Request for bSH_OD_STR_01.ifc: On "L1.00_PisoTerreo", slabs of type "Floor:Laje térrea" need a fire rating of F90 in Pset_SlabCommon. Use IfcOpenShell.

First a look at what the model holds.

```python
import ifcopenshell
import ifcopenshell.util.element

model = ifcopenshell.open("bSH_OD_STR_01.ifc")
print(model.schema)
storey = next(s for s in model.by_type("IfcBuildingStorey") if s.Name == "L1.00_PisoTerreo")
slabs = [e for e in ifcopenshell.util.element.get_decomposition(storey) if e.is_a("IfcSlab")]
seen = {}
for e in slabs:
    element_type = ifcopenshell.util.element.get_type(e)
    key = (element_type.Name if element_type != e and element_type else None, ifcopenshell.util.element.get_pset(e, "Pset_SlabCommon", "FireRating"))
    seen[key] = seen.get(key, 0) + 1
for (name, value), count in sorted(seen.items(), key=str):
    print(count, "x", name, "|", value)
```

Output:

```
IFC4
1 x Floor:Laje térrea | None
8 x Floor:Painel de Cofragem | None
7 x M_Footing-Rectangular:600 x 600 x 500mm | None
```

```python
import ifcopenshell
import ifcopenshell.api.pset
import ifcopenshell.util.element

model = ifcopenshell.open("bSH_OD_STR_01.ifc")

storey = next(s for s in model.by_type("IfcBuildingStorey") if s.Name == "L1.00_PisoTerreo")
slabs = [e for e in ifcopenshell.util.element.get_decomposition(storey) if e.is_a("IfcSlab")]

count = 0
for e in slabs:
    element_type = ifcopenshell.util.element.get_type(e)
    if element_type in (None, e) or element_type.Name != "Floor:Laje térrea":
        continue
    # add_pset returns the element's existing set when there is one.
    pset = ifcopenshell.api.pset.add_pset(model, product=e, name="Pset_SlabCommon")
    ifcopenshell.api.pset.edit_pset(model, pset=pset, properties={"FireRating": "F90"})
    count += 1

print(count, "slabs updated")

model.write("bSH_OD_STR_01_rev.ifc")
```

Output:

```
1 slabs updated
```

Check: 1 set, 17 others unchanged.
